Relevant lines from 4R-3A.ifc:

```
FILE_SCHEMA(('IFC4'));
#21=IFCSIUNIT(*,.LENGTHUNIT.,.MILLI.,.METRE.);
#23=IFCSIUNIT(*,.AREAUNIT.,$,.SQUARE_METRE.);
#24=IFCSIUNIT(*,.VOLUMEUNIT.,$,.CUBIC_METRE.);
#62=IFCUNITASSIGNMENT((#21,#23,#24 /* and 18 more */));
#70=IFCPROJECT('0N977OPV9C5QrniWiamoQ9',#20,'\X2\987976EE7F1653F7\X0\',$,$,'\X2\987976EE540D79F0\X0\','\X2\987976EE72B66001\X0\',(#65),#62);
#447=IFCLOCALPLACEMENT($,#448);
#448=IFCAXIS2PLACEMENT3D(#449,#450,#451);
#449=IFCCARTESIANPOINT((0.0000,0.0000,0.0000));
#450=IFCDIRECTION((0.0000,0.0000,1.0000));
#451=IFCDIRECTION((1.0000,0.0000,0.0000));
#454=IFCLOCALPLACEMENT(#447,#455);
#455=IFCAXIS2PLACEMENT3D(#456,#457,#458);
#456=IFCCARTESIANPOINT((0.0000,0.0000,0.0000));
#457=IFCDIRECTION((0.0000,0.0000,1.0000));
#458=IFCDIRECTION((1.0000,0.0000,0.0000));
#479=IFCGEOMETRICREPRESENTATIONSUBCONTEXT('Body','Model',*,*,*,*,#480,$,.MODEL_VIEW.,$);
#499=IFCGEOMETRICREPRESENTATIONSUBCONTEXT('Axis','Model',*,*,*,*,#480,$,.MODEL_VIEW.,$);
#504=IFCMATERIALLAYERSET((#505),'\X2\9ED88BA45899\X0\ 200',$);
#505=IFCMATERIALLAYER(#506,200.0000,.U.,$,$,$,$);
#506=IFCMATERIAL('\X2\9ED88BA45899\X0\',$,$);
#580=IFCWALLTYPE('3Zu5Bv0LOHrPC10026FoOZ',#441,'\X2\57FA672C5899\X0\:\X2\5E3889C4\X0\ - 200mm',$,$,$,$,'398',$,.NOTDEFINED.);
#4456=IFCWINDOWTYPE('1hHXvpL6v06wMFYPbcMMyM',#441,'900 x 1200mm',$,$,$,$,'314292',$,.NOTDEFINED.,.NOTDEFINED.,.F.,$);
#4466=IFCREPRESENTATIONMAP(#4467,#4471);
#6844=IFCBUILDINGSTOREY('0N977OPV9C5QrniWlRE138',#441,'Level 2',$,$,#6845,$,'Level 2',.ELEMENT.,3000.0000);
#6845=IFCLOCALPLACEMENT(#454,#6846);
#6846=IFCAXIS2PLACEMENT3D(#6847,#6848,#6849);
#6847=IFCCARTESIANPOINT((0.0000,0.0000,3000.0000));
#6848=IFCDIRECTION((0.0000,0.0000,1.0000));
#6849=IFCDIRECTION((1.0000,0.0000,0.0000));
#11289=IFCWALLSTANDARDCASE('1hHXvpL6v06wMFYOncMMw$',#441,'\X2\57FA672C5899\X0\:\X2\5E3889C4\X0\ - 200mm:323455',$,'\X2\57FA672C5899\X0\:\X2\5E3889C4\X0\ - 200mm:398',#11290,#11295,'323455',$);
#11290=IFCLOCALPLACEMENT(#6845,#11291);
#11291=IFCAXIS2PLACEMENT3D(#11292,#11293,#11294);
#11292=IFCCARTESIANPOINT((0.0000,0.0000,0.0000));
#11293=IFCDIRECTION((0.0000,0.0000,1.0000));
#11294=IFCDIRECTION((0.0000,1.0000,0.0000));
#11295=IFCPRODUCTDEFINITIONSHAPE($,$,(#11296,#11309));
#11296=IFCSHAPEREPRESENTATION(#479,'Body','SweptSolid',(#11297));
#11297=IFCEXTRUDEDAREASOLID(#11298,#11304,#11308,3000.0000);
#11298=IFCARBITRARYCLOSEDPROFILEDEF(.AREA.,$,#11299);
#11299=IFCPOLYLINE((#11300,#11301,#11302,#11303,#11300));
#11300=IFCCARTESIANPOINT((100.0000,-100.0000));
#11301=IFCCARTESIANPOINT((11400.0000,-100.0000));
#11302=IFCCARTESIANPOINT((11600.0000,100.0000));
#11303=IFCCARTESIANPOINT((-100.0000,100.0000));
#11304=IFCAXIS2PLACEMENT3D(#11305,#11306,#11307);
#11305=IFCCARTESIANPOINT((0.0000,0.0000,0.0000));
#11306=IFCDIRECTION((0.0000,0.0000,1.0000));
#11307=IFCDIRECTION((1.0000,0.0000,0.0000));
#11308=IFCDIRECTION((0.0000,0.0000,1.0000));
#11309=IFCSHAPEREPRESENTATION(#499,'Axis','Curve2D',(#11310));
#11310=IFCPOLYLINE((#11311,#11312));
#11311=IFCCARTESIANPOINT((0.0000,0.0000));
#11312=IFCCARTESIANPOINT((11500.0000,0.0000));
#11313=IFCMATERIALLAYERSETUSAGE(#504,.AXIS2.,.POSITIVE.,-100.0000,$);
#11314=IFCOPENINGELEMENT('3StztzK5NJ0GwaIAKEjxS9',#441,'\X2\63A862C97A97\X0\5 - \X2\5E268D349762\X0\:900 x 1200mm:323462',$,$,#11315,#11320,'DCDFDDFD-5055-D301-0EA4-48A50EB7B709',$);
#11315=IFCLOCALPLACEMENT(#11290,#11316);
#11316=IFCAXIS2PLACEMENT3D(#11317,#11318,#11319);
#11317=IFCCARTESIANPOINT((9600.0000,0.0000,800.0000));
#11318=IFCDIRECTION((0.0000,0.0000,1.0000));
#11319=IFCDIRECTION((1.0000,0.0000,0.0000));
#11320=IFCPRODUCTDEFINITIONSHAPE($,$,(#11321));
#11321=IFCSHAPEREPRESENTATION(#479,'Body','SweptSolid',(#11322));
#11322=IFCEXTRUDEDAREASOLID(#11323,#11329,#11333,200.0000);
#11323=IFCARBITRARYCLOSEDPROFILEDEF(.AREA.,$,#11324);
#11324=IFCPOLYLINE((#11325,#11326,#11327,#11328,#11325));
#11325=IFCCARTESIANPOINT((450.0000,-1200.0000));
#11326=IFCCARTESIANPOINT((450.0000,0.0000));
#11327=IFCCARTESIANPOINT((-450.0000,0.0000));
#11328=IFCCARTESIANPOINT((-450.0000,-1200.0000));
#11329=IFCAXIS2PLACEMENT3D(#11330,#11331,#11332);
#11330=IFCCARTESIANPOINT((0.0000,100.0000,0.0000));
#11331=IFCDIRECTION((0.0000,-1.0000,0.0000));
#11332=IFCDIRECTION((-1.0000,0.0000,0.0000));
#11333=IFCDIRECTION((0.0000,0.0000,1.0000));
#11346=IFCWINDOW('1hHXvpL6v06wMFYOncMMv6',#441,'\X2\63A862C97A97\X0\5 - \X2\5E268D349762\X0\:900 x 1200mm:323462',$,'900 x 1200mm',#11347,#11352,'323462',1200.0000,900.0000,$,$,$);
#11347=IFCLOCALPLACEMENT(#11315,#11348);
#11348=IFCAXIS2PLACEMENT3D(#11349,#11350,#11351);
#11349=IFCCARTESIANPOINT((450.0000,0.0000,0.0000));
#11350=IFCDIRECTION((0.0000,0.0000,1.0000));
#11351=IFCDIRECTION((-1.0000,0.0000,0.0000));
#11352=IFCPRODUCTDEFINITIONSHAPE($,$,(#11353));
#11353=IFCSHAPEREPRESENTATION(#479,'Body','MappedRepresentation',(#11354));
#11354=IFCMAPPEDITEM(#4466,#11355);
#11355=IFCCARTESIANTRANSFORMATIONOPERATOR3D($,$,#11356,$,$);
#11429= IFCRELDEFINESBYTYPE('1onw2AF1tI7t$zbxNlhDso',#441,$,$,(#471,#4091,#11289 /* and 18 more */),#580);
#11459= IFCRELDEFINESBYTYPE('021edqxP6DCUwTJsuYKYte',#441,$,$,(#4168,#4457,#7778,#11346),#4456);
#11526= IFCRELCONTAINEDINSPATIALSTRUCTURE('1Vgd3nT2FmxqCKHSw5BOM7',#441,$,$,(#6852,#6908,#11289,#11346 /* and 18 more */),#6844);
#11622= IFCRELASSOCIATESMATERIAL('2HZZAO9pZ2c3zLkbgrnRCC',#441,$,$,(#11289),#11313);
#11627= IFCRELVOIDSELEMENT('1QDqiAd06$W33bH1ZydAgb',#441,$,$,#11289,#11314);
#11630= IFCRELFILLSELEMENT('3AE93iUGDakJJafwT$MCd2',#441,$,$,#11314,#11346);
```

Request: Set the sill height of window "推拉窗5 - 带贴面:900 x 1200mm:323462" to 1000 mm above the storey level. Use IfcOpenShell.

```python
import numpy as np
import ifcopenshell
import ifcopenshell.api.geometry
import ifcopenshell.geom
import ifcopenshell.util.element
import ifcopenshell.util.placement
import ifcopenshell.util.shape
import ifcopenshell.util.unit

model = ifcopenshell.open("4R-3A.ifc")
unit_scale = ifcopenshell.util.unit.calculate_unit_scale(model)

window = model.by_guid("1hHXvpL6v06wMFYOncMMv6")
opening = window.FillsVoids[0].RelatingOpeningElement
storey = ifcopenshell.util.element.get_container(window, ifc_class="IfcBuildingStorey")
level = ifcopenshell.util.placement.get_local_placement(storey.ObjectPlacement)[2, 3]

# The opening's origin need not be at the sill, so measure its lowest point.
shape = ifcopenshell.geom.create_shape(ifcopenshell.geom.settings(), opening)
bottom = ifcopenshell.util.shape.get_shape_bottom_elevation(shape, shape.geometry) / unit_scale
dz = level + 1 / unit_scale - bottom

shift = np.array([0.0, 0.0, dz])
# The window is placed relative to its opening, so it follows when the opening moves.
matrix = ifcopenshell.util.placement.get_local_placement(opening.ObjectPlacement)
matrix[:3, 3] += shift
ifcopenshell.api.geometry.edit_object_placement(
    model, product=opening, matrix=matrix, is_si=False, should_transform_children=True
)

print(f"moved by {dz * unit_scale:+.3f} m")

model.write("4R-3A_updated.ifc")
```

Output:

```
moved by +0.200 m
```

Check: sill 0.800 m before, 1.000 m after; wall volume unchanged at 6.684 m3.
